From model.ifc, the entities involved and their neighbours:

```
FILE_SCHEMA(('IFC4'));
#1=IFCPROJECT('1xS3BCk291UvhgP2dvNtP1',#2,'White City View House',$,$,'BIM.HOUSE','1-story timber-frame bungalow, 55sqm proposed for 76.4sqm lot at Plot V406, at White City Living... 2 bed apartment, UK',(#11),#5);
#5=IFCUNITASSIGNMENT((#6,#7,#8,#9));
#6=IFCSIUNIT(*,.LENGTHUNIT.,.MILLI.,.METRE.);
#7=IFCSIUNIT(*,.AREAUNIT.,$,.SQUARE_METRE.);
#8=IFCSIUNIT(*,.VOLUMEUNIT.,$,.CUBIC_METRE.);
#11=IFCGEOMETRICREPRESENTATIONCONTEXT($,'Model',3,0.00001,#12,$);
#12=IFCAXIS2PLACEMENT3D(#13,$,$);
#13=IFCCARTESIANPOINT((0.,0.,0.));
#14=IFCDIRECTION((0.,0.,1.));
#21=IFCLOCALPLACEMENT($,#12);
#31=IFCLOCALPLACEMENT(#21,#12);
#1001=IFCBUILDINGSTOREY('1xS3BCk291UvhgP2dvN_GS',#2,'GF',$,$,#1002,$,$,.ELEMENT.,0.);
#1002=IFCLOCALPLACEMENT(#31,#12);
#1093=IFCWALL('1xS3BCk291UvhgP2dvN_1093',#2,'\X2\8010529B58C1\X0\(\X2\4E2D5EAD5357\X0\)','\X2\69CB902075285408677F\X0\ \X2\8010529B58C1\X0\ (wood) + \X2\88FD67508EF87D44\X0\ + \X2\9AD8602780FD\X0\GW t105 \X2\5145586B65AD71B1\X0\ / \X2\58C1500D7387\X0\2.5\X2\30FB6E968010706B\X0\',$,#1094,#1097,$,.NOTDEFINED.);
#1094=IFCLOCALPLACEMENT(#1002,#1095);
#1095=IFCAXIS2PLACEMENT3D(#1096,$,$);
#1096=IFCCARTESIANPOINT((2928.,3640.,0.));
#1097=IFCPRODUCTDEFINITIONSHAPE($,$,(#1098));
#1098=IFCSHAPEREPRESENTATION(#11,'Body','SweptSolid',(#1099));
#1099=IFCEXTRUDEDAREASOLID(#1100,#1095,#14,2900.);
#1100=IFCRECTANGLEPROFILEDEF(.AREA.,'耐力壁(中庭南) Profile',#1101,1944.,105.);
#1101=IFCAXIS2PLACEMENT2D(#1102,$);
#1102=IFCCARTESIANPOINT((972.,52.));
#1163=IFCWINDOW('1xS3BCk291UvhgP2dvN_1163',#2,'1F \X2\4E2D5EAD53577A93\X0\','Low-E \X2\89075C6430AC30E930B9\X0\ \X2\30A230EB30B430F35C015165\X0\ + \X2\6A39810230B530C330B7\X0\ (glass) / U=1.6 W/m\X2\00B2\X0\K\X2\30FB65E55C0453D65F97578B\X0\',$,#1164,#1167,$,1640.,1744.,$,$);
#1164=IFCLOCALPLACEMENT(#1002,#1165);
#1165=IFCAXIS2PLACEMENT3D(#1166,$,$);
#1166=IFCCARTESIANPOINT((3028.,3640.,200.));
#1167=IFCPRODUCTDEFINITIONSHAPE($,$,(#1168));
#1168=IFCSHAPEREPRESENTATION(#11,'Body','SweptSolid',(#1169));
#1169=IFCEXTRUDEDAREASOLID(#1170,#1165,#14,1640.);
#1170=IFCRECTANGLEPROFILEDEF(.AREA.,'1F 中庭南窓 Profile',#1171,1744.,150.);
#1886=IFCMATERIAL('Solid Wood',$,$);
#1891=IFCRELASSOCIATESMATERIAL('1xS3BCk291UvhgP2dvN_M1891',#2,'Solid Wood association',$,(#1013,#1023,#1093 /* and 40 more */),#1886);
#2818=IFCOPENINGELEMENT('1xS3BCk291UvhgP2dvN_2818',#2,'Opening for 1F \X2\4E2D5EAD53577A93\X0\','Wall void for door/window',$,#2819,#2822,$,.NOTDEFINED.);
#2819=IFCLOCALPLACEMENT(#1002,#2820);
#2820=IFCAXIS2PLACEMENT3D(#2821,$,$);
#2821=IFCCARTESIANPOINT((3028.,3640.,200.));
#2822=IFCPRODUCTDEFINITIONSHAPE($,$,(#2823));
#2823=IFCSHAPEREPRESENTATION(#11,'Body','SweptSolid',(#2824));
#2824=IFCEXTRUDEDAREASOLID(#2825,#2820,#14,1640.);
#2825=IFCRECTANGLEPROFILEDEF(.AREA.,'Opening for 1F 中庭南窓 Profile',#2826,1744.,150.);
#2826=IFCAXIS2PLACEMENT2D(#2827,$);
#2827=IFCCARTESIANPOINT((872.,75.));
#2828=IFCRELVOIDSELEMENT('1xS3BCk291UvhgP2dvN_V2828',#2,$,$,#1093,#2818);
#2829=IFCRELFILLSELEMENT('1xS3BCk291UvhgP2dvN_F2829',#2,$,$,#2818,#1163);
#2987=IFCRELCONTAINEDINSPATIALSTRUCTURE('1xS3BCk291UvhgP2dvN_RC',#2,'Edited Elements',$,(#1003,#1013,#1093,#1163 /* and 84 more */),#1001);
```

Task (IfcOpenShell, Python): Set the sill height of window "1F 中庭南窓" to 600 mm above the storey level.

```python
import numpy as np
import ifcopenshell
import ifcopenshell.api.geometry
import ifcopenshell.geom
import ifcopenshell.util.element
import ifcopenshell.util.placement
import ifcopenshell.util.shape
import ifcopenshell.util.unit

model = ifcopenshell.open("model.ifc")
unit_scale = ifcopenshell.util.unit.calculate_unit_scale(model)

window = model.by_guid("1xS3BCk291UvhgP2dvN_1163")
opening = window.FillsVoids[0].RelatingOpeningElement
storey = ifcopenshell.util.element.get_container(window, ifc_class="IfcBuildingStorey")
level = ifcopenshell.util.placement.get_local_placement(storey.ObjectPlacement)[2, 3]

# The opening's origin need not be at the sill, so measure its lowest point.
shape = ifcopenshell.geom.create_shape(ifcopenshell.geom.settings(), opening)
bottom = ifcopenshell.util.shape.get_shape_bottom_elevation(shape, shape.geometry) / unit_scale
dz = level + 0.6 / unit_scale - bottom

shift = np.array([0.0, 0.0, dz])
# The window is not placed relative to its opening, so move both.
for product in (opening, window):
    matrix = ifcopenshell.util.placement.get_local_placement(product.ObjectPlacement)
    matrix[:3, 3] += shift
    ifcopenshell.api.geometry.edit_object_placement(model, product=product, matrix=matrix, is_si=False)

print(f"moved by {dz * unit_scale:+.3f} m")

model.write("model-out.ifc")
```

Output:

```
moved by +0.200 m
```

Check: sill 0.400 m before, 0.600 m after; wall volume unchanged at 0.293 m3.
